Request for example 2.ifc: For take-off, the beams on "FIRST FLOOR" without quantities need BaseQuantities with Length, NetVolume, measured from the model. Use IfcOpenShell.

First a look at what the model holds.

```python
import ifcopenshell
import ifcopenshell.util.element
import ifcopenshell.util.unit

model = ifcopenshell.open("example 2.ifc")
print(model.schema)
for unit_type in ("LENGTHUNIT", "AREAUNIT", "VOLUMEUNIT"):
    print(unit_type, ifcopenshell.util.unit.calculate_unit_scale(model, unit_type))
storey = next(s for s in model.by_type("IfcBuildingStorey") if s.Name == "FIRST FLOOR")
beams = [e for e in ifcopenshell.util.element.get_decomposition(storey) if e.is_a("IfcBeam")]
for e in sorted(beams, key=lambda e: e.id()):
    print(e.id(), e.is_a(), e.Name, list(ifcopenshell.util.element.get_psets(e, qtos_only=True)), sep=" | ")
```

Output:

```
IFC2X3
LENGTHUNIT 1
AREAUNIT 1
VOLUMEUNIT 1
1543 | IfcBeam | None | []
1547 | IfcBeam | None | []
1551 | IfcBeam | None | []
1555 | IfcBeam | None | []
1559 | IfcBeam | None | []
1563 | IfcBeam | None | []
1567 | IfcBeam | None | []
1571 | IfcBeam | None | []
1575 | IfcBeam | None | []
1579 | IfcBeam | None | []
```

```python
import ifcopenshell
import ifcopenshell.api.pset
import ifcopenshell.geom
import ifcopenshell.util.element
import ifcopenshell.util.shape
import ifcopenshell.util.unit

model = ifcopenshell.open("example 2.ifc")
unit_scale = ifcopenshell.util.unit.calculate_unit_scale(model)
volume_scale = ifcopenshell.util.unit.calculate_unit_scale(model, "VOLUMEUNIT")
settings = ifcopenshell.geom.settings()

storey = next(s for s in model.by_type("IfcBuildingStorey") if s.Name == "FIRST FLOOR")
beams = [e for e in ifcopenshell.util.element.get_decomposition(storey) if e.is_a("IfcBeam")]

for e in sorted(beams, key=lambda e: e.id()):
    if ifcopenshell.util.element.get_psets(e, qtos_only=True, should_inherit=False):
        continue
    # Geometry comes back in metres, in the element's own axes.
    shape = ifcopenshell.geom.create_shape(settings, e)
    values = {
        "Length": ifcopenshell.util.shape.get_max_xyz(shape.geometry) / unit_scale,
        "NetVolume": ifcopenshell.util.shape.get_volume(shape.geometry) / volume_scale,
    }
    qto = ifcopenshell.api.pset.add_qto(model, product=e, name="BaseQuantities")
    ifcopenshell.api.pset.edit_qto(model, qto=qto, properties=values)
    print(e.id(), {k: round(v, 3) for k, v in values.items()})

model.write("example 2_rev.ifc")
```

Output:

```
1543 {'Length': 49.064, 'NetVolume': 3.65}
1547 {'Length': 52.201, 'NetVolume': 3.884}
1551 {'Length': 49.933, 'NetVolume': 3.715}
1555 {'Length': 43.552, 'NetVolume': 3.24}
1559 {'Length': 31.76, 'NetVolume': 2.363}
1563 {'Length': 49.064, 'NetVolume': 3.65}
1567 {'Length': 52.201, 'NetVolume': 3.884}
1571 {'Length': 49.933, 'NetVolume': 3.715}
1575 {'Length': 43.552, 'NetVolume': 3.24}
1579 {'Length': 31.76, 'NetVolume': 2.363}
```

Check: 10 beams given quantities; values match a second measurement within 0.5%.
